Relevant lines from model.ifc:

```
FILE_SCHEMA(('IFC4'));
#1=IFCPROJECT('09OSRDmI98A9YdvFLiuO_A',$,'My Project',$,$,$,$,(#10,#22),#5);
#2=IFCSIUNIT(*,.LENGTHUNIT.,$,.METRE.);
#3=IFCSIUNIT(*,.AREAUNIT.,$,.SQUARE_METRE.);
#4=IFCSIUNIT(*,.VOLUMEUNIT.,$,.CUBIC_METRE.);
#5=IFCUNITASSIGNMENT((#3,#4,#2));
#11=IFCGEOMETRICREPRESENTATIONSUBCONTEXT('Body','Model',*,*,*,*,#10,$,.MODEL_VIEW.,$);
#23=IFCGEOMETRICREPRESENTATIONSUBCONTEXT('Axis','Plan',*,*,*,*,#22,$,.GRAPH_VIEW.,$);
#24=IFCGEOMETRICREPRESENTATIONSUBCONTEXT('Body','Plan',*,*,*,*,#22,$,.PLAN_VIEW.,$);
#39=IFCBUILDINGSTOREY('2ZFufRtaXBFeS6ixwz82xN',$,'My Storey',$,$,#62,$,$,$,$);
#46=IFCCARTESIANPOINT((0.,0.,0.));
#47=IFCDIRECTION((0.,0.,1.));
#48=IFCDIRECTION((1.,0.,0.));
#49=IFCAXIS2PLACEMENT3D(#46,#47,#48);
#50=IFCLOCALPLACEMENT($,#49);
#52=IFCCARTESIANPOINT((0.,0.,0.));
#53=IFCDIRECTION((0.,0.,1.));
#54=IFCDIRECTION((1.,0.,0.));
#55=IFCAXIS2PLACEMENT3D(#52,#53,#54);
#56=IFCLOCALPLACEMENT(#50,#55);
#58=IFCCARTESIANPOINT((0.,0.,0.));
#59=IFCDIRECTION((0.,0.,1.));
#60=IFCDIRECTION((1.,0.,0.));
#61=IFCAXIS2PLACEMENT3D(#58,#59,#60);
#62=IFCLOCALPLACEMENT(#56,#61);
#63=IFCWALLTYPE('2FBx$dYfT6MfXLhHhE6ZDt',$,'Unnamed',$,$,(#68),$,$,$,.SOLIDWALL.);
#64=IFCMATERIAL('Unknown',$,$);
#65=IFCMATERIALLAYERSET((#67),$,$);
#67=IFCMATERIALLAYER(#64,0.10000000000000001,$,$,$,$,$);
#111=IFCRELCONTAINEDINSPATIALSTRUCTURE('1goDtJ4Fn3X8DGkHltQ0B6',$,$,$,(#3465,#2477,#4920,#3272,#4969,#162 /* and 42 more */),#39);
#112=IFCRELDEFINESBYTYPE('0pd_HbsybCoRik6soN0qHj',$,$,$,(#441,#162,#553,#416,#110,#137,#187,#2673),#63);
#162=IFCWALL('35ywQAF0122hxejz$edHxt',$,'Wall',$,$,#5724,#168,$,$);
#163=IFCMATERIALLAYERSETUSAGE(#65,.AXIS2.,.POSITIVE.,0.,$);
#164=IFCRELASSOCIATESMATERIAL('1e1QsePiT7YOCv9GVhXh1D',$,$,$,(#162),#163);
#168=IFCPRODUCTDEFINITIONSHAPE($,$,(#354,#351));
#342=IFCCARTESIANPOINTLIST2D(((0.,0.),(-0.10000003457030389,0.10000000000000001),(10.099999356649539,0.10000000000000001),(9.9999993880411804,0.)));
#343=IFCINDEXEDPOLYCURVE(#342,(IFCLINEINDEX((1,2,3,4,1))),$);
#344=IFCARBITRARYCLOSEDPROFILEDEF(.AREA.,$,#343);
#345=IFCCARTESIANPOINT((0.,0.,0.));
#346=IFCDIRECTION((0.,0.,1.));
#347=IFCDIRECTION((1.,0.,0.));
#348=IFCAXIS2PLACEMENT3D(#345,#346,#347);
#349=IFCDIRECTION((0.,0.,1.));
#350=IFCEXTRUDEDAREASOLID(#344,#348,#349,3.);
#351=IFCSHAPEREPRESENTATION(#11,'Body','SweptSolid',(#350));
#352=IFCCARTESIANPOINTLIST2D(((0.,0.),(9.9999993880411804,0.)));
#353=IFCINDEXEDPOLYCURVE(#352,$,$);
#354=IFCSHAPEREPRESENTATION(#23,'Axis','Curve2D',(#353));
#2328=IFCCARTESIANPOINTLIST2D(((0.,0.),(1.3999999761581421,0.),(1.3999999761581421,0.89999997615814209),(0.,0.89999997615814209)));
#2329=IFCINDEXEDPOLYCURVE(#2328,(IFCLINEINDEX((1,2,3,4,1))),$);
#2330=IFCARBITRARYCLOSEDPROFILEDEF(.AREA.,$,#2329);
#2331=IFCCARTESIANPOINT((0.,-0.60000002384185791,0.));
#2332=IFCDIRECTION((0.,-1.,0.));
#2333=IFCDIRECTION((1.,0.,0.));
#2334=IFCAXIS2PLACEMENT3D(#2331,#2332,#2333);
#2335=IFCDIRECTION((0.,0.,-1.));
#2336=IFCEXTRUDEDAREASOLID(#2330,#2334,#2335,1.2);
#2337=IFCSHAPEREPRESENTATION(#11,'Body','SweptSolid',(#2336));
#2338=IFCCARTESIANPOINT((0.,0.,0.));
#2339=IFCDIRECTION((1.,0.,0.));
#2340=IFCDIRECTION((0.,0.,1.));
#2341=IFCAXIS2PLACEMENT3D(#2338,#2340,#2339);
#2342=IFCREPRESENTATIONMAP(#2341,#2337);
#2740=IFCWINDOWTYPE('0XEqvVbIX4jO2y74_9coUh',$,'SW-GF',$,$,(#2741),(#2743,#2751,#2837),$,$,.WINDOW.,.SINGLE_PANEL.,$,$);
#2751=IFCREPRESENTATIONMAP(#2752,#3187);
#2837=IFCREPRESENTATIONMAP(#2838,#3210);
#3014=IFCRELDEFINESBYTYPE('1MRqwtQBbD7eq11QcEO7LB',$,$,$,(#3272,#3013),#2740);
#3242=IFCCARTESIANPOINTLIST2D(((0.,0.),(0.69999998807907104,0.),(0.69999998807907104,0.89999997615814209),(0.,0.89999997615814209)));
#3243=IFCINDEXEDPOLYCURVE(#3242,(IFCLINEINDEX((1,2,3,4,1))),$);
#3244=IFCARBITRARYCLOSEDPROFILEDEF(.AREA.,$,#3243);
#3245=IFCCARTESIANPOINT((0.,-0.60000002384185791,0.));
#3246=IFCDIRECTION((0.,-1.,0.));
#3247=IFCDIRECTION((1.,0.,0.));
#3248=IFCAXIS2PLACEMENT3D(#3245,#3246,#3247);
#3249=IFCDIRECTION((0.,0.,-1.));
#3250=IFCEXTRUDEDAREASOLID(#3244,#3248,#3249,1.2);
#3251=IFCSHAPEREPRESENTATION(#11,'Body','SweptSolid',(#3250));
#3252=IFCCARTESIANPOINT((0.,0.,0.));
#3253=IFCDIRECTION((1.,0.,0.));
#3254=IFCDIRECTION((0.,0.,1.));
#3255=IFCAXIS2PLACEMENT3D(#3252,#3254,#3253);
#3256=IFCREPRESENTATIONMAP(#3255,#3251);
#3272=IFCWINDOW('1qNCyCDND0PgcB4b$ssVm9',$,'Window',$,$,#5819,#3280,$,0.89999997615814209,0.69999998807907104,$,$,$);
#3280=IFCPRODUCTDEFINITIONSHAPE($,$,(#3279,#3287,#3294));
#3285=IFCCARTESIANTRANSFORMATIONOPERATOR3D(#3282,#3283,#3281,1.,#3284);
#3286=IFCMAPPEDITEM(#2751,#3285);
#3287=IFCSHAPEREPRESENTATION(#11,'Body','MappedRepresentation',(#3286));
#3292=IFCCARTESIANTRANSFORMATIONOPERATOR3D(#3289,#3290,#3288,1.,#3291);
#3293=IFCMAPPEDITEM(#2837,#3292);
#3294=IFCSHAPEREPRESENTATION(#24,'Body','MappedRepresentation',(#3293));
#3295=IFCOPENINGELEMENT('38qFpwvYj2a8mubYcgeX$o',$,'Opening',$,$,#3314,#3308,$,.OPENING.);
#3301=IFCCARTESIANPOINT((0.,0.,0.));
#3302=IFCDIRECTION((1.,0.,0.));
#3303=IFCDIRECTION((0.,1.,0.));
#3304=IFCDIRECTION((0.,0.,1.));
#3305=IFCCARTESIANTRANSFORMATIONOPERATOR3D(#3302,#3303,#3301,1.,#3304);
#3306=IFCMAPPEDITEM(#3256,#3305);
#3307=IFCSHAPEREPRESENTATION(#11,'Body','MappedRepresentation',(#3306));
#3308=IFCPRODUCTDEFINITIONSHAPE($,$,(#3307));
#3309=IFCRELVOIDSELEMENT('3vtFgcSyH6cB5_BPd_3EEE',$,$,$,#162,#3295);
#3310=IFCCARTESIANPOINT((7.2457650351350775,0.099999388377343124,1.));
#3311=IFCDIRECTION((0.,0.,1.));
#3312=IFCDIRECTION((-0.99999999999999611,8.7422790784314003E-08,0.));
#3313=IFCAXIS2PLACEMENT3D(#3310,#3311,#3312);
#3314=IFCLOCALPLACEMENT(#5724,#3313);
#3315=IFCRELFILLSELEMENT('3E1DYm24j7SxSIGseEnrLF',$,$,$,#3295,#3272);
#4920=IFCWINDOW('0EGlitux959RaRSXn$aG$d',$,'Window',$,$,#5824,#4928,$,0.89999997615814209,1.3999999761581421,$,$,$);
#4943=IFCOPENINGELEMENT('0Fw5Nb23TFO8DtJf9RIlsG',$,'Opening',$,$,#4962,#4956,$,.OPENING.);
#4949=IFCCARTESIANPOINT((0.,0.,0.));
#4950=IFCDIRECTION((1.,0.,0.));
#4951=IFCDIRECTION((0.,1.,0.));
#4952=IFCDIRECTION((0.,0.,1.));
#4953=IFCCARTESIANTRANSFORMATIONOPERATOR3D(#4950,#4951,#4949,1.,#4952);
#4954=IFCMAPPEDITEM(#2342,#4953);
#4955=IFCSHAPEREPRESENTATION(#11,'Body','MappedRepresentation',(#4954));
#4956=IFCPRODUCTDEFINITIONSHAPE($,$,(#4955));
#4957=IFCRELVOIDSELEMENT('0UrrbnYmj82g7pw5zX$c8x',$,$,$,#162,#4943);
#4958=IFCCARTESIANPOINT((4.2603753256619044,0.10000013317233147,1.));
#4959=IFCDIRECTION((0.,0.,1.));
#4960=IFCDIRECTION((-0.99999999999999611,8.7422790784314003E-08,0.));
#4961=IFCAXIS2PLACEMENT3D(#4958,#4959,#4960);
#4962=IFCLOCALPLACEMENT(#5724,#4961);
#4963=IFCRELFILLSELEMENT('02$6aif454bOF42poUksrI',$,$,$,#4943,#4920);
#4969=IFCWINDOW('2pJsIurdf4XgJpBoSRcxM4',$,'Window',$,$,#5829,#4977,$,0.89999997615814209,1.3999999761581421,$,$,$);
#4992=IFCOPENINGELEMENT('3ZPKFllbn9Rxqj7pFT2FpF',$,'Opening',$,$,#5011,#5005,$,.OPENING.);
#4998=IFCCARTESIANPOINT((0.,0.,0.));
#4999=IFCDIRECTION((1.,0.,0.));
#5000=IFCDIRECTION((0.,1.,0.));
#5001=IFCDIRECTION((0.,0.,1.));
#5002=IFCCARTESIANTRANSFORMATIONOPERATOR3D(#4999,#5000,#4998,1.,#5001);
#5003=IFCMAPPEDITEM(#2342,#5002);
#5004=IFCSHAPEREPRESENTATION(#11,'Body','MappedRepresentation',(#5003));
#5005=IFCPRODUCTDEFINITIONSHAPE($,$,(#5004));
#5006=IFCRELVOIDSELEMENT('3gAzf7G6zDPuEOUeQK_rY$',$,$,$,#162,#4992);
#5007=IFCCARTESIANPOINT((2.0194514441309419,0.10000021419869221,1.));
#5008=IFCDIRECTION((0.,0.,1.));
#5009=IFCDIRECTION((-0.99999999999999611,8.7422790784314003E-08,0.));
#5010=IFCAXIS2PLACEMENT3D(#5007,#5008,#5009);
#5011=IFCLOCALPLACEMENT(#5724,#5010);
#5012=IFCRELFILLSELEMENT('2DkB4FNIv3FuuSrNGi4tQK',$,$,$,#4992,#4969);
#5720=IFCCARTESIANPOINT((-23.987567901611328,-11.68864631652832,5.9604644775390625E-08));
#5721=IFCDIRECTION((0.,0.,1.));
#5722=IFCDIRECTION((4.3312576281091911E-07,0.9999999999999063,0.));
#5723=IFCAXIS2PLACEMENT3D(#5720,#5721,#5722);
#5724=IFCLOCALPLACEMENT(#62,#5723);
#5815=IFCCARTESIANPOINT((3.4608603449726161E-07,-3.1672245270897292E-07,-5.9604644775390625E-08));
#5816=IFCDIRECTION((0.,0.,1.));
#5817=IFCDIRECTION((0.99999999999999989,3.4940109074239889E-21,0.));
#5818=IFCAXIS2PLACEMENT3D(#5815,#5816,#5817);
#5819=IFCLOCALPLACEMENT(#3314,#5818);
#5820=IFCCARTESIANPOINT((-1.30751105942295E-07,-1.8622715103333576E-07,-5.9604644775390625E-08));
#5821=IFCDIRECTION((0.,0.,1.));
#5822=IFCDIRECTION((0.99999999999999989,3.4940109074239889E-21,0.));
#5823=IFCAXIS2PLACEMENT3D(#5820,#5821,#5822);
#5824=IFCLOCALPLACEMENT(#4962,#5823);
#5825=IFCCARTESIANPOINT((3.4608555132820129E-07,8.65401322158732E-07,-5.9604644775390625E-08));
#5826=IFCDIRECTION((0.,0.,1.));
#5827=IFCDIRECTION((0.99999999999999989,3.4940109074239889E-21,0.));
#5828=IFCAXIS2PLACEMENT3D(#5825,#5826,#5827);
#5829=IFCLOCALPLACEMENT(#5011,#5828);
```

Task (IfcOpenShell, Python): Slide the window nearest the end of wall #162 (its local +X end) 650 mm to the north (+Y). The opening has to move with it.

```python
import ifcopenshell
import ifcopenshell.api.geometry
import ifcopenshell.util.placement

model = ifcopenshell.open("model.ifc")

window = model.by_guid("1qNCyCDND0PgcB4b$ssVm9")
opening = window.FillsVoids[0].RelatingOpeningElement
wall = opening.VoidsElements[0].RelatingBuildingElement

wall_matrix = ifcopenshell.util.placement.get_local_placement(wall.ObjectPlacement)
shift = wall_matrix[:3, 0] * 0.65
before = ifcopenshell.util.placement.get_local_placement(window.ObjectPlacement)[:3, 3].copy()

# The window is placed relative to its opening, so it follows when the opening moves.
matrix = ifcopenshell.util.placement.get_local_placement(opening.ObjectPlacement)
matrix[:3, 3] += shift
ifcopenshell.api.geometry.edit_object_placement(
    model, product=opening, matrix=matrix, is_si=False, should_transform_children=True
)

after = ifcopenshell.util.placement.get_local_placement(window.ObjectPlacement)[:3, 3]
print("window moved by", (after - before).round(3) + 0.0)

model.write("model_rev.ifc")
```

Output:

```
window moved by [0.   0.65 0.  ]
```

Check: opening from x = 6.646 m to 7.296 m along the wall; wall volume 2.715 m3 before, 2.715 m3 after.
